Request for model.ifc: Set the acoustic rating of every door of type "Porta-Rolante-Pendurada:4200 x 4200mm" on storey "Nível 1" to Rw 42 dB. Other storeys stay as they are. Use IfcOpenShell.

First a look at what the model holds.

```python
import ifcopenshell
import ifcopenshell.util.element

model = ifcopenshell.open("model.ifc")
print(model.schema)
storey = next(s for s in model.by_type("IfcBuildingStorey") if s.Name == "Nível 1")
doors = [e for e in ifcopenshell.util.element.get_decomposition(storey) if e.is_a("IfcDoor")]
seen = {}
for e in doors:
    element_type = ifcopenshell.util.element.get_type(e)
    key = (element_type.Name if element_type != e and element_type else None, ifcopenshell.util.element.get_pset(e, "Pset_DoorCommon", "AcousticRating"))
    seen[key] = seen.get(key, 0) + 1
for (name, value), count in sorted(seen.items(), key=str):
    print(count, "x", name, "|", value)
```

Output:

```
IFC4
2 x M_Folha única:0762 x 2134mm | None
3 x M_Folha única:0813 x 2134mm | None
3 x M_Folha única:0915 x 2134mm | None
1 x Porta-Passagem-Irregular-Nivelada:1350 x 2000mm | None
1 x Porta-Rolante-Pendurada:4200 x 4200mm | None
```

```python
import ifcopenshell
import ifcopenshell.api.pset
import ifcopenshell.util.element

model = ifcopenshell.open("model.ifc")

storey = next(s for s in model.by_type("IfcBuildingStorey") if s.Name == "Nível 1")
doors = [e for e in ifcopenshell.util.element.get_decomposition(storey) if e.is_a("IfcDoor")]

count = 0
for e in doors:
    element_type = ifcopenshell.util.element.get_type(e)
    if element_type in (None, e) or element_type.Name != "Porta-Rolante-Pendurada:4200 x 4200mm":
        continue
    # add_pset returns the element's existing set when there is one.
    pset = ifcopenshell.api.pset.add_pset(model, product=e, name="Pset_DoorCommon")
    ifcopenshell.api.pset.edit_pset(model, pset=pset, properties={"AcousticRating": "Rw 42 dB"})
    count += 1

print(count, "doors updated")

model.write("model_rev.ifc")
```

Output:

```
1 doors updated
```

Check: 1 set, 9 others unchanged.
